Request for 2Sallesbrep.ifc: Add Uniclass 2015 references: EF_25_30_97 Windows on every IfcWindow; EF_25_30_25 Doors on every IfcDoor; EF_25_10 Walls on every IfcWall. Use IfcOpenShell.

First a look at what the model holds.

```python
import ifcopenshell

model = ifcopenshell.open("2Sallesbrep.ifc")
print(model.schema)
print("classifications:", [c.Name for c in model.by_type("IfcClassification")])
for ifc_class in ("IfcDoor", "IfcRoof", "IfcStair", "IfcWall", "IfcWindow"):
    print(ifc_class, len(model.by_type(ifc_class)))
```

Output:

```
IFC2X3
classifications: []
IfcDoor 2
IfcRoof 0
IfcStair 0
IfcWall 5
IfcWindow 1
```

```python
import ifcopenshell
import ifcopenshell.api.classification

model = ifcopenshell.open("2Sallesbrep.ifc")

# IFC2X3 requires Source and Edition and has no link from the project to the system.
system = model.create_entity("IfcClassification", Source="NBS", Edition="2015", Name="Uniclass 2015")

codes = {
    "IfcWindow": ("EF_25_30_97", "Windows"),
    "IfcDoor": ("EF_25_30_25", "Doors"),
    "IfcWall": ("EF_25_10", "Walls"),
}
for ifc_class, (code, name) in codes.items():
    products = model.by_type(ifc_class)
    ifcopenshell.api.classification.add_reference(
        model, products=products, classification=system, identification=code, name=name
    )
    print(code, len(products))

model.write("2Sallesbrep_rev.ifc")
```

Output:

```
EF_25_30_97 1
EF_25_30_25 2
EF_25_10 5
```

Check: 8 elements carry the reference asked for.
